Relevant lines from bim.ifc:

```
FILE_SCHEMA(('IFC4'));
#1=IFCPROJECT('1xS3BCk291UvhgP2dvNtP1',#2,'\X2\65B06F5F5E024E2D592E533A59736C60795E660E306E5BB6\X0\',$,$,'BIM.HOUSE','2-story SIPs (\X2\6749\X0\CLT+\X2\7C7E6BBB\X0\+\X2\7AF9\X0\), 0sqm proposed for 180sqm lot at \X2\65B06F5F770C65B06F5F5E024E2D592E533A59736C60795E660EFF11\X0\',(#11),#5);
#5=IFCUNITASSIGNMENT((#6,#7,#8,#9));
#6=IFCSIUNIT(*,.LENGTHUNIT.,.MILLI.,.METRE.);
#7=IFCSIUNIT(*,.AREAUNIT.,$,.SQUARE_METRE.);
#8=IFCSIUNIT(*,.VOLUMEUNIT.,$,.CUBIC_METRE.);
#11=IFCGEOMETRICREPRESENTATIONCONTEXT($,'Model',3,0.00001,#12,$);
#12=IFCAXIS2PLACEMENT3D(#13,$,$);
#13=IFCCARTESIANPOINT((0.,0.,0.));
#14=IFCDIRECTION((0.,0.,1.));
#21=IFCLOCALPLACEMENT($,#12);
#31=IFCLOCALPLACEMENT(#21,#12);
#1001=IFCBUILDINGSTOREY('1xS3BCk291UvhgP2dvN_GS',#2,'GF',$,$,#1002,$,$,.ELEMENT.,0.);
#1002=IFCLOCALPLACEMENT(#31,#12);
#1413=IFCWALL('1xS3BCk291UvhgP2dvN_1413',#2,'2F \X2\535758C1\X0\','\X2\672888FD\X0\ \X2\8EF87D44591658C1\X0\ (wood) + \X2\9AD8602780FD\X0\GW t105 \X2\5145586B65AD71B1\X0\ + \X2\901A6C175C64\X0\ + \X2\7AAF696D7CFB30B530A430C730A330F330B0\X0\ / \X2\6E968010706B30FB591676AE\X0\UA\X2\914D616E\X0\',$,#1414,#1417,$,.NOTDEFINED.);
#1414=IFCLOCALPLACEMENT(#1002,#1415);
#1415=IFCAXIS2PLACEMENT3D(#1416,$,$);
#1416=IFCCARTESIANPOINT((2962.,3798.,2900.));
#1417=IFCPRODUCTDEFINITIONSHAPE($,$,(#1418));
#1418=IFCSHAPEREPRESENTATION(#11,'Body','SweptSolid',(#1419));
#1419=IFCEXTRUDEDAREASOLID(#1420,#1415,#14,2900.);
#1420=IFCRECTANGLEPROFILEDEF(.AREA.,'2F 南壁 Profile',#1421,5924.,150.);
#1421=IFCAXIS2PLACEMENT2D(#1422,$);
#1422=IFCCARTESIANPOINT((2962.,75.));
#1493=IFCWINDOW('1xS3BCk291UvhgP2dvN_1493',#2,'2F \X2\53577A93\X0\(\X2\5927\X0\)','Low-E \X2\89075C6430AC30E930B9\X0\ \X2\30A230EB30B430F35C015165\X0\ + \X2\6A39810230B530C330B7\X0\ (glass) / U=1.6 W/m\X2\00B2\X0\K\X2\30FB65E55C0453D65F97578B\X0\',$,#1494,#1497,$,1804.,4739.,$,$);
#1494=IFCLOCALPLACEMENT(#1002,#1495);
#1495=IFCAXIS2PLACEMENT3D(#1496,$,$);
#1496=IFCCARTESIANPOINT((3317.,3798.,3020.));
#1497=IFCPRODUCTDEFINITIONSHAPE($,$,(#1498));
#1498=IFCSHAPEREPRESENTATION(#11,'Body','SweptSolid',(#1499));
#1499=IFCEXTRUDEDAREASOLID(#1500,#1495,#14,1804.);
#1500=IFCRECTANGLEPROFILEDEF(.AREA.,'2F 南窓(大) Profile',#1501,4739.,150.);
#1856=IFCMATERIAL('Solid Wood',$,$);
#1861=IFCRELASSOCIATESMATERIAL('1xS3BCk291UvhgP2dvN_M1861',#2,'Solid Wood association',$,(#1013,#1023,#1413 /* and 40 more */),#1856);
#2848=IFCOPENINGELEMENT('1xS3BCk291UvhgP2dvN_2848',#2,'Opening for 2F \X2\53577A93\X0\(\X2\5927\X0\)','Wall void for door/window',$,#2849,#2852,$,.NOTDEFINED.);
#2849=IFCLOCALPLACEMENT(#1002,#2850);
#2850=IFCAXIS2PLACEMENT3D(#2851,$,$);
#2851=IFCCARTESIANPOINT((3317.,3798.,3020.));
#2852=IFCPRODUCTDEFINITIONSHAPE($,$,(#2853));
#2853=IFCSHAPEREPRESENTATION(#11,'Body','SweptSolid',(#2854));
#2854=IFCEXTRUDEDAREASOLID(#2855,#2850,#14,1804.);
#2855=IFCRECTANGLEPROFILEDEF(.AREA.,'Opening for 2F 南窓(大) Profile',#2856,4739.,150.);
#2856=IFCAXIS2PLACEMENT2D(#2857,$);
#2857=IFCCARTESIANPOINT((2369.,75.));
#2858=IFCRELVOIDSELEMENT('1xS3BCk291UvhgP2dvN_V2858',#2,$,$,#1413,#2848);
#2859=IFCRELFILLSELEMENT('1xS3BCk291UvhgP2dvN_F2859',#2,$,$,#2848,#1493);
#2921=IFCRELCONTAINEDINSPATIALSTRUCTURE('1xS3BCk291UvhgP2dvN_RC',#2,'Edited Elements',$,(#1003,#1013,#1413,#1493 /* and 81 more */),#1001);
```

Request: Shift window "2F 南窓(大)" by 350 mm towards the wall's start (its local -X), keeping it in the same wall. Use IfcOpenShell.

```python
import ifcopenshell
import ifcopenshell.api.geometry
import ifcopenshell.util.placement
import ifcopenshell.util.unit

model = ifcopenshell.open("bim.ifc")
unit_scale = ifcopenshell.util.unit.calculate_unit_scale(model)

window = model.by_guid("1xS3BCk291UvhgP2dvN_1493")
opening = window.FillsVoids[0].RelatingOpeningElement
wall = opening.VoidsElements[0].RelatingBuildingElement

wall_matrix = ifcopenshell.util.placement.get_local_placement(wall.ObjectPlacement)
shift = wall_matrix[:3, 0] * -0.35 / unit_scale
before = ifcopenshell.util.placement.get_local_placement(window.ObjectPlacement)[:3, 3].copy()

# The window is not placed relative to its opening, so move both.
for product in (opening, window):
    matrix = ifcopenshell.util.placement.get_local_placement(product.ObjectPlacement)
    matrix[:3, 3] += shift
    ifcopenshell.api.geometry.edit_object_placement(model, product=product, matrix=matrix, is_si=False)

after = ifcopenshell.util.placement.get_local_placement(window.ObjectPlacement)[:3, 3]
print("window moved by", (after - before).round(3) + 0.0)

model.write("bim_rev.ifc")
```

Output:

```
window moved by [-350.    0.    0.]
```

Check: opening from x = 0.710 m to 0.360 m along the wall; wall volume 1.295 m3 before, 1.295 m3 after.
